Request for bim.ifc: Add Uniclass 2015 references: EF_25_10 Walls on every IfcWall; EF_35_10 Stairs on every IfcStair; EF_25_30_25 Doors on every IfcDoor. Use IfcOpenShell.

First a look at what the model holds.

```python
import ifcopenshell

model = ifcopenshell.open("bim.ifc")
print(model.schema)
print("classifications:", [c.Name for c in model.by_type("IfcClassification")])
for ifc_class in ("IfcDoor", "IfcRoof", "IfcStair", "IfcWall", "IfcWindow"):
    print(ifc_class, len(model.by_type(ifc_class)))
```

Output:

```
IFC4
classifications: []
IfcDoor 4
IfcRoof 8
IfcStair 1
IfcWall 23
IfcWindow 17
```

```python
import ifcopenshell
import ifcopenshell.api.classification

model = ifcopenshell.open("bim.ifc")

system = ifcopenshell.api.classification.add_classification(model, classification="Uniclass 2015")

codes = {
    "IfcWall": ("EF_25_10", "Walls"),
    "IfcStair": ("EF_35_10", "Stairs"),
    "IfcDoor": ("EF_25_30_25", "Doors"),
}
for ifc_class, (code, name) in codes.items():
    products = model.by_type(ifc_class)
    ifcopenshell.api.classification.add_reference(
        model, products=products, classification=system, identification=code, name=name
    )
    print(code, len(products))

model.write("bim_rev.ifc")
```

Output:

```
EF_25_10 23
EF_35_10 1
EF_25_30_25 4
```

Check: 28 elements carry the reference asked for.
